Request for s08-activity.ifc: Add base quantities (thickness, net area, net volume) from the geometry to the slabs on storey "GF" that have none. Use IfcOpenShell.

First a look at what the model holds.

```python
import ifcopenshell
import ifcopenshell.util.element
import ifcopenshell.util.unit

model = ifcopenshell.open("s08-activity.ifc")
print(model.schema)
for unit_type in ("LENGTHUNIT", "AREAUNIT", "VOLUMEUNIT"):
    print(unit_type, ifcopenshell.util.unit.calculate_unit_scale(model, unit_type))
storey = next(s for s in model.by_type("IfcBuildingStorey") if s.Name == "GF")
slabs = [e for e in ifcopenshell.util.element.get_decomposition(storey) if e.is_a("IfcSlab")]
for e in sorted(slabs, key=lambda e: e.id()):
    print(e.id(), e.is_a(), e.Name, list(ifcopenshell.util.element.get_psets(e, qtos_only=True)), sep=" | ")
```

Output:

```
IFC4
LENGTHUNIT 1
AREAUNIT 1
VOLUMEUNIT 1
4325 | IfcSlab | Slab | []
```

```python
import ifcopenshell
import ifcopenshell.api.pset
import ifcopenshell.geom
import ifcopenshell.util.element
import ifcopenshell.util.shape
import ifcopenshell.util.unit

model = ifcopenshell.open("s08-activity.ifc")
unit_scale = ifcopenshell.util.unit.calculate_unit_scale(model)
area_scale = ifcopenshell.util.unit.calculate_unit_scale(model, "AREAUNIT")
volume_scale = ifcopenshell.util.unit.calculate_unit_scale(model, "VOLUMEUNIT")
settings = ifcopenshell.geom.settings()

storey = next(s for s in model.by_type("IfcBuildingStorey") if s.Name == "GF")
slabs = [e for e in ifcopenshell.util.element.get_decomposition(storey) if e.is_a("IfcSlab")]

for e in sorted(slabs, key=lambda e: e.id()):
    if ifcopenshell.util.element.get_psets(e, qtos_only=True, should_inherit=False):
        continue
    # Geometry comes back in metres, in the element's own axes.
    shape = ifcopenshell.geom.create_shape(settings, e)
    values = {
        "Width": ifcopenshell.util.shape.get_z(shape.geometry) / unit_scale,
        "NetArea": ifcopenshell.util.shape.get_footprint_area(shape.geometry) / area_scale,
        "NetVolume": ifcopenshell.util.shape.get_volume(shape.geometry) / volume_scale,
    }
    qto = ifcopenshell.api.pset.add_qto(model, product=e, name="Qto_SlabBaseQuantities")
    ifcopenshell.api.pset.edit_qto(model, qto=qto, properties=values)
    print(e.id(), {k: round(v, 3) for k, v in values.items()})

model.write("s08-activity-out.ifc")
```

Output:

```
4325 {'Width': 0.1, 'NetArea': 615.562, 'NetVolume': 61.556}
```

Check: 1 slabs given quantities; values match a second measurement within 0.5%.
